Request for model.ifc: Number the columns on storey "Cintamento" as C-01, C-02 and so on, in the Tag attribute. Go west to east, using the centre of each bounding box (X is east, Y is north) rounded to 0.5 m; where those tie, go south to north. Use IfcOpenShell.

First a look at what the model holds.

```python
import ifcopenshell
import ifcopenshell.util.element
import ifcopenshell.util.placement

model = ifcopenshell.open("model.ifc")
print(model.schema)
storey = next(s for s in model.by_type("IfcBuildingStorey") if s.Name == "Cintamento")
columns = [e for e in ifcopenshell.util.element.get_decomposition(storey) if e.is_a("IfcColumn")]
for e in sorted(columns, key=lambda e: e.id()):
    origin = ifcopenshell.util.placement.get_local_placement(e.ObjectPlacement)[:3, 3]
    print(e.id(), e.Tag, e.Name, origin.round(2) + 0.0, sep=" | ")
```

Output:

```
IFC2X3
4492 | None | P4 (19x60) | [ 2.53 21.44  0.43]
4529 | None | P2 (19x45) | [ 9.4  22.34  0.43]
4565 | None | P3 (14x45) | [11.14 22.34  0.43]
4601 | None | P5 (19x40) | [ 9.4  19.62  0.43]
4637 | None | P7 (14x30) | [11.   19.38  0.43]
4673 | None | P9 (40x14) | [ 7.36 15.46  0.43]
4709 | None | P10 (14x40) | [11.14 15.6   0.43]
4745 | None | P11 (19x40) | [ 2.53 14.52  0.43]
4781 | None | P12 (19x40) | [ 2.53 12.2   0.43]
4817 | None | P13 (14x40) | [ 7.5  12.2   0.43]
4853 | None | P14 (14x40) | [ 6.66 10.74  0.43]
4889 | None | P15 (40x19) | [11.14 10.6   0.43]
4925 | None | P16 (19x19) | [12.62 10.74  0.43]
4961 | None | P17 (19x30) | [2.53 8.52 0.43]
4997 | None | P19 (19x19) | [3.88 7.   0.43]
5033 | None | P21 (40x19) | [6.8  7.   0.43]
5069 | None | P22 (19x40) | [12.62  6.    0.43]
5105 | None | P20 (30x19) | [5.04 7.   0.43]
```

```python
import ifcopenshell
import ifcopenshell.geom
import ifcopenshell.util.element
import ifcopenshell.util.shape

model = ifcopenshell.open("model.ifc")
settings = ifcopenshell.geom.settings()
settings.set("use-world-coords", True)


def centre(element):
    shape = ifcopenshell.geom.create_shape(settings, element)
    return ifcopenshell.util.shape.get_bbox_centroid(shape.geometry)


storey = next(s for s in model.by_type("IfcBuildingStorey") if s.Name == "Cintamento")
columns = [e for e in ifcopenshell.util.element.get_decomposition(storey) if e.is_a("IfcColumn")]

# Insertion points can sit at a corner or the storey origin, so sort by the geometry (in metres).
centres = {e: centre(e) for e in columns}
columns.sort(key=lambda e: (round(centres[e][0] / 0.5), centres[e][1]))

for i, e in enumerate(columns, start=1):
    number = f"C-{i:02d}"
    e.Tag = number
    print(e.id(), number)

model.write("model_updated.ifc")
```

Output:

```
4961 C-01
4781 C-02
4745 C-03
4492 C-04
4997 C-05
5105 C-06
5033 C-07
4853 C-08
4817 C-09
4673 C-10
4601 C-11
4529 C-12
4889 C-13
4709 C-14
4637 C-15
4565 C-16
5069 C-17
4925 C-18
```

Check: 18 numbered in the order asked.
